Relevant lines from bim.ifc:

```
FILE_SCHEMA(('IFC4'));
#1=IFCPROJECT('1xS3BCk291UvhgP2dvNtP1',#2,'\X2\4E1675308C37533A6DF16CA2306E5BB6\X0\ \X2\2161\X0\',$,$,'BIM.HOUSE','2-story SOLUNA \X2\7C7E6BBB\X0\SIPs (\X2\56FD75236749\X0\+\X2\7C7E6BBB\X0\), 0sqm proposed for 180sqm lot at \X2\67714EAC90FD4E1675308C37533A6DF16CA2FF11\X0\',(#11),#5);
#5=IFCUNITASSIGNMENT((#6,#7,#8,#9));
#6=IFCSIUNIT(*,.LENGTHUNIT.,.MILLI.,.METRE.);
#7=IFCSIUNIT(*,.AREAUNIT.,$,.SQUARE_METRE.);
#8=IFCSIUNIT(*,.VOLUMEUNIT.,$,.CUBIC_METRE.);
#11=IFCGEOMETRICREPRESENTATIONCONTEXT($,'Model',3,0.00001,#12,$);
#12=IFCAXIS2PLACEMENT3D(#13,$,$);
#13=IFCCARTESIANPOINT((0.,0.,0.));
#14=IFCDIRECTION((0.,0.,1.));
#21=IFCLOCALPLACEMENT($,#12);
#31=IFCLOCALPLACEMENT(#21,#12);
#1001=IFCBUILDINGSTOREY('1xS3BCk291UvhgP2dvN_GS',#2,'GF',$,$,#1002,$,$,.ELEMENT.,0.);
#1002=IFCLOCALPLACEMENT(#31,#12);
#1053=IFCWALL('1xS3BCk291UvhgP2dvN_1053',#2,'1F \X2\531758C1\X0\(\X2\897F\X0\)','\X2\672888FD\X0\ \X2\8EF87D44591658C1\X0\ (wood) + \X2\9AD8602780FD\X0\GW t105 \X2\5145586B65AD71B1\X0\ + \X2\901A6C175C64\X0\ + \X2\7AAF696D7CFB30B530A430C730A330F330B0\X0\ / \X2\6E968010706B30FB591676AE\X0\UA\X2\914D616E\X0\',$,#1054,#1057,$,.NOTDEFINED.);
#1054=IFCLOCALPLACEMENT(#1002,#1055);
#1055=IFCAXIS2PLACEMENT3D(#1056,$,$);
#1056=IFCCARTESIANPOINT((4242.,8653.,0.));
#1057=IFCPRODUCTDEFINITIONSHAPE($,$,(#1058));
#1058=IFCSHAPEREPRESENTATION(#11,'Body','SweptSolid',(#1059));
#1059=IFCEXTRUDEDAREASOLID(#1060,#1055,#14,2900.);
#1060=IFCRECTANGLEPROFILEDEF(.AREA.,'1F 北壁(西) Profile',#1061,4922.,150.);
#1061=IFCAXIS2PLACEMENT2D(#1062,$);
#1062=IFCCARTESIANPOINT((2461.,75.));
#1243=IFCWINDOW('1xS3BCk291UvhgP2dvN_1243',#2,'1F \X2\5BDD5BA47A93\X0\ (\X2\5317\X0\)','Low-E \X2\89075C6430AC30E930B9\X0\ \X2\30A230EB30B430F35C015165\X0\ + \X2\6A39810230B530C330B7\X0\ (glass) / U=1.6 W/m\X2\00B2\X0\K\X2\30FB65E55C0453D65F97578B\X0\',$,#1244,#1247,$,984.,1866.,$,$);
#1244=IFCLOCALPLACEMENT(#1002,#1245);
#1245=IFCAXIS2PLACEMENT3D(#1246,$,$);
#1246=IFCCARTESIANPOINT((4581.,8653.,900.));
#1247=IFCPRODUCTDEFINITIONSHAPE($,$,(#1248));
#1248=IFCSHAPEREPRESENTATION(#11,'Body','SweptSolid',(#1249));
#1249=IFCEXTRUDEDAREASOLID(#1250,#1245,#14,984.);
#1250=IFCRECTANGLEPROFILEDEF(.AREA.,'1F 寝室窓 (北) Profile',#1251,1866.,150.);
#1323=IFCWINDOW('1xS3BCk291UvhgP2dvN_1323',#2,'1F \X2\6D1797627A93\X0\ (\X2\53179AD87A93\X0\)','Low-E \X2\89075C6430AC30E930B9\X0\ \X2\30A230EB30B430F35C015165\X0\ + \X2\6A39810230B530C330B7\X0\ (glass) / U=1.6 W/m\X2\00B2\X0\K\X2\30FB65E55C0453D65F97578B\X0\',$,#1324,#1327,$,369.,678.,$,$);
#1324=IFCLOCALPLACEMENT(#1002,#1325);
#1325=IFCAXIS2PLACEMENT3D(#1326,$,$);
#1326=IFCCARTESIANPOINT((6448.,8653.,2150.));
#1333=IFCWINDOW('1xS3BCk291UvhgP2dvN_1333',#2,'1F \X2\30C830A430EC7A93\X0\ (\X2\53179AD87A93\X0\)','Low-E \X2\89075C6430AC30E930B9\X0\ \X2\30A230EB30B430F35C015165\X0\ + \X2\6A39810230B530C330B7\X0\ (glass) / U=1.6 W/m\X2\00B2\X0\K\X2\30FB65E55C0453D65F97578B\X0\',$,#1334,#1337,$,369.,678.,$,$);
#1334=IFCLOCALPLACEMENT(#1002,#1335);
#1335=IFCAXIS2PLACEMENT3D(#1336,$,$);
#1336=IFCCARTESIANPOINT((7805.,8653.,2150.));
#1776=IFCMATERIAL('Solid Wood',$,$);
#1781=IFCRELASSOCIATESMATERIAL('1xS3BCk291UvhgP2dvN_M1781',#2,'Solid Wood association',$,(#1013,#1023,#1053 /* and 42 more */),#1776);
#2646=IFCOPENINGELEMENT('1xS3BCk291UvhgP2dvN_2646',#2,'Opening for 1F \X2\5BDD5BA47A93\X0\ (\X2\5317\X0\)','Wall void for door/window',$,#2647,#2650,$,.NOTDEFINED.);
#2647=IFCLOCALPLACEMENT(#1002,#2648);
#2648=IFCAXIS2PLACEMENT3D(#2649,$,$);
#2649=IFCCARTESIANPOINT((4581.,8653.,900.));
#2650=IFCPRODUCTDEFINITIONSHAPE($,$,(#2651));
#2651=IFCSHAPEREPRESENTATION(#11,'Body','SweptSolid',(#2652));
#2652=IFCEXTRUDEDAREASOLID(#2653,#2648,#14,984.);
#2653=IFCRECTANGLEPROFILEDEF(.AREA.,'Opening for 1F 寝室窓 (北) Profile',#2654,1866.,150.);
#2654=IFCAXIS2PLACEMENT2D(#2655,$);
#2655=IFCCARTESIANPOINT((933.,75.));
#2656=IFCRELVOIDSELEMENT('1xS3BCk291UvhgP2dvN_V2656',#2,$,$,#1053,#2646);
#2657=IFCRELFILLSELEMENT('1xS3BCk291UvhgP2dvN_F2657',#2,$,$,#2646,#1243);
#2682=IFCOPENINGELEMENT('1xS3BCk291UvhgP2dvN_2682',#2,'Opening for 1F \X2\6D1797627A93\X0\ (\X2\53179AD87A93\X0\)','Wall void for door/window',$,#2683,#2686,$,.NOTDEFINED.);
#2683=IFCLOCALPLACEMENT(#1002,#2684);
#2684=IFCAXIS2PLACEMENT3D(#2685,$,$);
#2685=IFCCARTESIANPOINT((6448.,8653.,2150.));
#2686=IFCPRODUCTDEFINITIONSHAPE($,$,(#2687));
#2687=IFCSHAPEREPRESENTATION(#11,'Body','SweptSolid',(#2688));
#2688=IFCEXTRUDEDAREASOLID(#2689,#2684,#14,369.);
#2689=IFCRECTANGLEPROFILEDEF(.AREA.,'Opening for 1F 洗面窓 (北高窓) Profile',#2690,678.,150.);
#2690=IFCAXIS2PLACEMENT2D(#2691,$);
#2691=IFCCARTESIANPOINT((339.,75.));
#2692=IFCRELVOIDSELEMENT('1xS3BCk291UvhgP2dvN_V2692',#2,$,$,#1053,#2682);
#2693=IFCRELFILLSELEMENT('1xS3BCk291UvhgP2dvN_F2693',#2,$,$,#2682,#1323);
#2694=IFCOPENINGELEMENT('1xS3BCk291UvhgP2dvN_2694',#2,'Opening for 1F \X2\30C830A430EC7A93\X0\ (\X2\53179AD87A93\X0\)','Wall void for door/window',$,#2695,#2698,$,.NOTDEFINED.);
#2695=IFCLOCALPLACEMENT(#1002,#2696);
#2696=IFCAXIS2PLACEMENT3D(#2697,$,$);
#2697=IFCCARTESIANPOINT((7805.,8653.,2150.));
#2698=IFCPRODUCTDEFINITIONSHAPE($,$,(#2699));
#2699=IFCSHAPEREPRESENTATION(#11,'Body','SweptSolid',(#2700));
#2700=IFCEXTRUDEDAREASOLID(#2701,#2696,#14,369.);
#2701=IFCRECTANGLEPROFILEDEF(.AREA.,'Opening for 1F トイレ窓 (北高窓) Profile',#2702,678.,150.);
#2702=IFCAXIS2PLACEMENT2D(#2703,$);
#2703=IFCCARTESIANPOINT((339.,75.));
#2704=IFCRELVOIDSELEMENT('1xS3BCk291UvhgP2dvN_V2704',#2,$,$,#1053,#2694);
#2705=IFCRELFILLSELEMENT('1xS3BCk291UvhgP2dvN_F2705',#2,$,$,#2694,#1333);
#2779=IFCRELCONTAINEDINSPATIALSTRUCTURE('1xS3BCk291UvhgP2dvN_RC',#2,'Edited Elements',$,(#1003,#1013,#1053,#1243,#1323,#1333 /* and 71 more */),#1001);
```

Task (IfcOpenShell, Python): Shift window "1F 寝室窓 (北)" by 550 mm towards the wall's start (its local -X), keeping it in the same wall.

```python
import ifcopenshell
import ifcopenshell.api.geometry
import ifcopenshell.util.placement

model = ifcopenshell.open("bim.ifc")

window = model.by_guid("1xS3BCk291UvhgP2dvN_1243")
opening = window.FillsVoids[0].RelatingOpeningElement
wall = opening.VoidsElements[0].RelatingBuildingElement

wall_matrix = ifcopenshell.util.placement.get_local_placement(wall.ObjectPlacement)
shift = wall_matrix[:3, 0] * -550.0
before = ifcopenshell.util.placement.get_local_placement(window.ObjectPlacement)[:3, 3].copy()

# The window is not placed relative to its opening, so move both.
for product in (opening, window):
    matrix = ifcopenshell.util.placement.get_local_placement(product.ObjectPlacement)
    matrix[:3, 3] += shift
    ifcopenshell.api.geometry.edit_object_placement(model, product=product, matrix=matrix, is_si=False)

after = ifcopenshell.util.placement.get_local_placement(window.ObjectPlacement)[:3, 3]
print("window moved by", (after - before).round(3) + 0.0)

model.write("bim_edited.ifc")
```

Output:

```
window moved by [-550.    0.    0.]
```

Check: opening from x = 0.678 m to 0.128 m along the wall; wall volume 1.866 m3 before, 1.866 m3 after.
